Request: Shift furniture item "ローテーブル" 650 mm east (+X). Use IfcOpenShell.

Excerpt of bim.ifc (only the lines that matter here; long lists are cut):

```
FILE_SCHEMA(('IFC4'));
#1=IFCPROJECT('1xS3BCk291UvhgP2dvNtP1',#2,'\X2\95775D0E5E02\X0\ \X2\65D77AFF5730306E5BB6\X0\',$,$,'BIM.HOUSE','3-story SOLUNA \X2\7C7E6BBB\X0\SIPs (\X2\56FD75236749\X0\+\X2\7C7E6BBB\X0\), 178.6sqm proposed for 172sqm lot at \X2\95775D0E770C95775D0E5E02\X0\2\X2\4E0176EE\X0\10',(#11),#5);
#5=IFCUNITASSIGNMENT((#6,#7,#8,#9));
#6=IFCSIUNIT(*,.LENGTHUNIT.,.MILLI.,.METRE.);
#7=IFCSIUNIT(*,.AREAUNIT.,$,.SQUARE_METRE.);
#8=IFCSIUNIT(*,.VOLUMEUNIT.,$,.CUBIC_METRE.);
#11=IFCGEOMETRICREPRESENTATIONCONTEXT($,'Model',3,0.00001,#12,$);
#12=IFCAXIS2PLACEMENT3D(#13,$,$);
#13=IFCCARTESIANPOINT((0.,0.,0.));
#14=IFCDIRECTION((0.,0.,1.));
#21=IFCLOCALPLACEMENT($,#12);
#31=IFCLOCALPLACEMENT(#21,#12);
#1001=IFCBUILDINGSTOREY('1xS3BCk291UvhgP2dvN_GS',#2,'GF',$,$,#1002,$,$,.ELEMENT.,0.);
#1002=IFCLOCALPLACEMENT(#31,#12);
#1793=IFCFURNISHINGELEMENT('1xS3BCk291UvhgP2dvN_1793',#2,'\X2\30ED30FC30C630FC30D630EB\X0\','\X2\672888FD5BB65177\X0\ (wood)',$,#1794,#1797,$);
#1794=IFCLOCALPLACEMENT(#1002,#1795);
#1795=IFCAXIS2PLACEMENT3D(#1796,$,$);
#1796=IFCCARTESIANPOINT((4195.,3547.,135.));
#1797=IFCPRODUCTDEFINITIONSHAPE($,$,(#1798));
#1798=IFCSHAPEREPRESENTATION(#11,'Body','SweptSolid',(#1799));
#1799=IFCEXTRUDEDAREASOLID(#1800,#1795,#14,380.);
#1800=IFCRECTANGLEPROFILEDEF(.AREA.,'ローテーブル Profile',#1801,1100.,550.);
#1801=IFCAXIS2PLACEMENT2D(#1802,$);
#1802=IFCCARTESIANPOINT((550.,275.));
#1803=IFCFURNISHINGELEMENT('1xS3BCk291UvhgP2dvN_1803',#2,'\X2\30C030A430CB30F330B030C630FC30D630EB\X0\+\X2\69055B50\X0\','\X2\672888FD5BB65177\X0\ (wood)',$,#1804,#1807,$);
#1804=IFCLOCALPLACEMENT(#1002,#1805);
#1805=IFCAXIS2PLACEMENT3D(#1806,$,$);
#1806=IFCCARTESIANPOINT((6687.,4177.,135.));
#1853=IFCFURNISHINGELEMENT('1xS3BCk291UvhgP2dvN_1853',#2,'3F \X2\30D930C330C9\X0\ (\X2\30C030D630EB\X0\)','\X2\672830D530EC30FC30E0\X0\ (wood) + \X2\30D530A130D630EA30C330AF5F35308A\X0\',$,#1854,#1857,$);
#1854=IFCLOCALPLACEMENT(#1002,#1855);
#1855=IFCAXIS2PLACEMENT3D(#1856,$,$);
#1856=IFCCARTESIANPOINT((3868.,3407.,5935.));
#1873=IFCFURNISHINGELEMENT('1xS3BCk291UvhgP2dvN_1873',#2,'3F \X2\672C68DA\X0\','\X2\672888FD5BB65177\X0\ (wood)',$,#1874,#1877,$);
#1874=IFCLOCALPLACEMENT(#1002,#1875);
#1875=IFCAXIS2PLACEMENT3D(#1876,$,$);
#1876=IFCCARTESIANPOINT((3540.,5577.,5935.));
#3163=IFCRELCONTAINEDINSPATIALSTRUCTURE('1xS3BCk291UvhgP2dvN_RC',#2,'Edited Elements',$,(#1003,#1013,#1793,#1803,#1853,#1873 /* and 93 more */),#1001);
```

```python
import ifcopenshell
import ifcopenshell.api.geometry
import ifcopenshell.util.placement

model = ifcopenshell.open("bim.ifc")

item = model.by_guid("1xS3BCk291UvhgP2dvN_1793")
matrix = ifcopenshell.util.placement.get_local_placement(item.ObjectPlacement)
matrix[0, 3] += 650.0
ifcopenshell.api.geometry.edit_object_placement(model, product=item, matrix=matrix, is_si=False)

print(ifcopenshell.util.placement.get_local_placement(item.ObjectPlacement).round(3) + 0.0)

model.write("bim_updated.ifc")
```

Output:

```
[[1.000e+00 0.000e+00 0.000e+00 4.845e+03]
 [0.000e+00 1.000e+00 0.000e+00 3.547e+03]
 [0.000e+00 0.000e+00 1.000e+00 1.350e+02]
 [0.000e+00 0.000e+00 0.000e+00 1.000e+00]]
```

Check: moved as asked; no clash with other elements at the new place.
